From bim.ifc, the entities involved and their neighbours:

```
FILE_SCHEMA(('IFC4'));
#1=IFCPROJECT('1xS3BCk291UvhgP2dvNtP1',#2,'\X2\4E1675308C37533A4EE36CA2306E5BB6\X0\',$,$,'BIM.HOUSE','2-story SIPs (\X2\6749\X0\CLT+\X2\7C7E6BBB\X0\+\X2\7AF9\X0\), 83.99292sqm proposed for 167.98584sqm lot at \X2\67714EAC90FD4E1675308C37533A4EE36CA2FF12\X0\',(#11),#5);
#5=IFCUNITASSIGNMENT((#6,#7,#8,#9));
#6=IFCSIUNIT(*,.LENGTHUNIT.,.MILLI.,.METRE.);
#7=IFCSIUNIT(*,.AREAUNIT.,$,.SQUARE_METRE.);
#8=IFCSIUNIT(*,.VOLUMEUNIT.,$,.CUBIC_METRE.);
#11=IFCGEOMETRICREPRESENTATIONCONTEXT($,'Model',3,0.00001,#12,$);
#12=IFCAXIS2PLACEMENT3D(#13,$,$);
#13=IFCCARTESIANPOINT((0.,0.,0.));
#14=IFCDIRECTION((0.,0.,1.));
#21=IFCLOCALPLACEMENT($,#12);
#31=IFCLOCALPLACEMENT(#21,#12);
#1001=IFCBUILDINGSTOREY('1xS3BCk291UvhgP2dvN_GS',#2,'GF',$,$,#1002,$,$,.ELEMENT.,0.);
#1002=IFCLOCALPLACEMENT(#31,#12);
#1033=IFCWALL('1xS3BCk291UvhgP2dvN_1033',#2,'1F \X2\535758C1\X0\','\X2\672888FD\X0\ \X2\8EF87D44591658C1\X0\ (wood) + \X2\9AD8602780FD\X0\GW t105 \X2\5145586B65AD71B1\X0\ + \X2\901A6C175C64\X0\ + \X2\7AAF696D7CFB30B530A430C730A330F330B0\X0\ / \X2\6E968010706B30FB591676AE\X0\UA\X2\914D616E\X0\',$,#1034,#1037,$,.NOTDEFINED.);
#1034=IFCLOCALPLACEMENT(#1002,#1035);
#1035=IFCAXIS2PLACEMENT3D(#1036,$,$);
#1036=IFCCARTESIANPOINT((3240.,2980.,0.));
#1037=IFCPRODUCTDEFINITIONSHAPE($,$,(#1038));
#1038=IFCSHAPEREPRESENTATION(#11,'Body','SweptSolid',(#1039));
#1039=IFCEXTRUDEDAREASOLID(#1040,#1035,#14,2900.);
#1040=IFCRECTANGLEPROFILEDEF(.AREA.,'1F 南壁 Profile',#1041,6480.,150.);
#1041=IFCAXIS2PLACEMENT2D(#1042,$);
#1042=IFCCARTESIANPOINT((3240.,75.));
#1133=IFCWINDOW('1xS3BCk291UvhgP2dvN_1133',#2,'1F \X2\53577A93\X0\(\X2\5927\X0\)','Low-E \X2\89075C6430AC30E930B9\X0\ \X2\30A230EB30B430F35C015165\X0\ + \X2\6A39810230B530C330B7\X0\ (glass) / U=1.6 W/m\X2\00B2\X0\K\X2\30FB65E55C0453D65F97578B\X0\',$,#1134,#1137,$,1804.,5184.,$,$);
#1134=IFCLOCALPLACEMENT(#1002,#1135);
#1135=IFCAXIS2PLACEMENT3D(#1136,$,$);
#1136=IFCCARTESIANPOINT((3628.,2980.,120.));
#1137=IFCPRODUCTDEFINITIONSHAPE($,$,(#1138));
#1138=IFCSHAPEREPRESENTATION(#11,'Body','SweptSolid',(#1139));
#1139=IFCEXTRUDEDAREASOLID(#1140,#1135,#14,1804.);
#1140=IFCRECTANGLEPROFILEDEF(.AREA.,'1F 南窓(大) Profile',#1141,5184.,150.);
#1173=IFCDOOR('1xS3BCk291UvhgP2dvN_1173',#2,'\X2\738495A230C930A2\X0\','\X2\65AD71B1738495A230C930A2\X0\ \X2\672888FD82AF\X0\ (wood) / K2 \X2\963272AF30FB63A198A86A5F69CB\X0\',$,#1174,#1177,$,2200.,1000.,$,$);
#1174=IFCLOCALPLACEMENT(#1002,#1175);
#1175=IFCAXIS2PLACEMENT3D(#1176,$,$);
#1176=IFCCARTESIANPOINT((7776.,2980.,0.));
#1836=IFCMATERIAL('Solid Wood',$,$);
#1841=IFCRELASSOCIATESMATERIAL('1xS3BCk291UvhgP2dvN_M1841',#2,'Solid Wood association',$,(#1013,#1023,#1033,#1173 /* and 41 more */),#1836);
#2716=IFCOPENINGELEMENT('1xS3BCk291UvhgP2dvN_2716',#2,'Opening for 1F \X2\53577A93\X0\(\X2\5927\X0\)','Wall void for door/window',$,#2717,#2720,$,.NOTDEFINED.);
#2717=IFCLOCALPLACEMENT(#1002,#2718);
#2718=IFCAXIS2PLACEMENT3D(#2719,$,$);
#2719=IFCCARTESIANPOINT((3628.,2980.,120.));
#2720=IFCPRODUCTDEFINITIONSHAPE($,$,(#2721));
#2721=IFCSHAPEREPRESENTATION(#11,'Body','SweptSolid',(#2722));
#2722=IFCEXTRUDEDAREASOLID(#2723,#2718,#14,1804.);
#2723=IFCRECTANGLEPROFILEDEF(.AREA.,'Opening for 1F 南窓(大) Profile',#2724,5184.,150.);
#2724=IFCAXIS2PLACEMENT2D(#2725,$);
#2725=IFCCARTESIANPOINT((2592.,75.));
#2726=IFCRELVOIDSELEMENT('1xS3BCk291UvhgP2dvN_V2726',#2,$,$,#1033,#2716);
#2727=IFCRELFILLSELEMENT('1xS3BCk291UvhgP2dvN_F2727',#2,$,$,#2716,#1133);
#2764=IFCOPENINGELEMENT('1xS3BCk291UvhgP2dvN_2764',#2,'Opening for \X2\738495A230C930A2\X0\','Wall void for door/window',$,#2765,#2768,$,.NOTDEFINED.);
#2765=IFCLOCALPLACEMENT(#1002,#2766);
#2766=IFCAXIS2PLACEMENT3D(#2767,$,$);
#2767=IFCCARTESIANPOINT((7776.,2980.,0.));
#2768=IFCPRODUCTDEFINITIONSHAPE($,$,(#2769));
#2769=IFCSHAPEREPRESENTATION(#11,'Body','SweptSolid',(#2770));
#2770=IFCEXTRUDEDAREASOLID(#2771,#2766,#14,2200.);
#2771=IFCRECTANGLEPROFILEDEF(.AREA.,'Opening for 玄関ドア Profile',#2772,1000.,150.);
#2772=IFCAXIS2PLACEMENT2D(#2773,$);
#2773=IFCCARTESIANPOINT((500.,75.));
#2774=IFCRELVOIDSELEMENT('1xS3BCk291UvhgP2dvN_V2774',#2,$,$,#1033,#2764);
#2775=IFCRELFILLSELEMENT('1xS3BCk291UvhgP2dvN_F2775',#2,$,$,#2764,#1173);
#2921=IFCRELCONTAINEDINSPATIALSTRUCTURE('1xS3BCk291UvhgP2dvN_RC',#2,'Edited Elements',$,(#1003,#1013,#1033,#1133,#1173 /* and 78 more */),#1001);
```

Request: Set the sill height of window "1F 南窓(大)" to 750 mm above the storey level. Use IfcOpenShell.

```python
import numpy as np
import ifcopenshell
import ifcopenshell.api.geometry
import ifcopenshell.geom
import ifcopenshell.util.element
import ifcopenshell.util.placement
import ifcopenshell.util.shape
import ifcopenshell.util.unit

model = ifcopenshell.open("bim.ifc")
unit_scale = ifcopenshell.util.unit.calculate_unit_scale(model)

window = model.by_guid("1xS3BCk291UvhgP2dvN_1133")
opening = window.FillsVoids[0].RelatingOpeningElement
storey = ifcopenshell.util.element.get_container(window, ifc_class="IfcBuildingStorey")
level = ifcopenshell.util.placement.get_local_placement(storey.ObjectPlacement)[2, 3]

# The opening's origin need not be at the sill, so measure its lowest point.
shape = ifcopenshell.geom.create_shape(ifcopenshell.geom.settings(), opening)
bottom = ifcopenshell.util.shape.get_shape_bottom_elevation(shape, shape.geometry) / unit_scale
dz = level + 0.75 / unit_scale - bottom

shift = np.array([0.0, 0.0, dz])
# The window is not placed relative to its opening, so move both.
for product in (opening, window):
    matrix = ifcopenshell.util.placement.get_local_placement(product.ObjectPlacement)
    matrix[:3, 3] += shift
    ifcopenshell.api.geometry.edit_object_placement(model, product=product, matrix=matrix, is_si=False)

print(f"moved by {dz * unit_scale:+.3f} m")

model.write("bim_updated.ifc")
```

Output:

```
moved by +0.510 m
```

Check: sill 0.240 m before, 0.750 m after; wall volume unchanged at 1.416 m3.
